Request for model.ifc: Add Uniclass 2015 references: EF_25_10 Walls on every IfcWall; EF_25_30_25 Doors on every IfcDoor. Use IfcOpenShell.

First a look at what the model holds.

```python
import ifcopenshell

model = ifcopenshell.open("model.ifc")
print(model.schema)
print("classifications:", [c.Name for c in model.by_type("IfcClassification")])
for ifc_class in ("IfcDoor", "IfcRoof", "IfcStair", "IfcWall", "IfcWindow"):
    print(ifc_class, len(model.by_type(ifc_class)))
```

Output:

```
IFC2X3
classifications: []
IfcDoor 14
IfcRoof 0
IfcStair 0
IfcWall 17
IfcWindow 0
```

```python
import ifcopenshell
import ifcopenshell.api.classification

model = ifcopenshell.open("model.ifc")

# IFC2X3 requires Source and Edition and has no link from the project to the system.
system = model.create_entity("IfcClassification", Source="NBS", Edition="2015", Name="Uniclass 2015")

codes = {
    "IfcWall": ("EF_25_10", "Walls"),
    "IfcDoor": ("EF_25_30_25", "Doors"),
}
for ifc_class, (code, name) in codes.items():
    products = model.by_type(ifc_class)
    ifcopenshell.api.classification.add_reference(
        model, products=products, classification=system, identification=code, name=name
    )
    print(code, len(products))

model.write("model-out.ifc")
```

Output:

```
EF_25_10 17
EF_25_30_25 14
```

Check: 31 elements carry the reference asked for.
